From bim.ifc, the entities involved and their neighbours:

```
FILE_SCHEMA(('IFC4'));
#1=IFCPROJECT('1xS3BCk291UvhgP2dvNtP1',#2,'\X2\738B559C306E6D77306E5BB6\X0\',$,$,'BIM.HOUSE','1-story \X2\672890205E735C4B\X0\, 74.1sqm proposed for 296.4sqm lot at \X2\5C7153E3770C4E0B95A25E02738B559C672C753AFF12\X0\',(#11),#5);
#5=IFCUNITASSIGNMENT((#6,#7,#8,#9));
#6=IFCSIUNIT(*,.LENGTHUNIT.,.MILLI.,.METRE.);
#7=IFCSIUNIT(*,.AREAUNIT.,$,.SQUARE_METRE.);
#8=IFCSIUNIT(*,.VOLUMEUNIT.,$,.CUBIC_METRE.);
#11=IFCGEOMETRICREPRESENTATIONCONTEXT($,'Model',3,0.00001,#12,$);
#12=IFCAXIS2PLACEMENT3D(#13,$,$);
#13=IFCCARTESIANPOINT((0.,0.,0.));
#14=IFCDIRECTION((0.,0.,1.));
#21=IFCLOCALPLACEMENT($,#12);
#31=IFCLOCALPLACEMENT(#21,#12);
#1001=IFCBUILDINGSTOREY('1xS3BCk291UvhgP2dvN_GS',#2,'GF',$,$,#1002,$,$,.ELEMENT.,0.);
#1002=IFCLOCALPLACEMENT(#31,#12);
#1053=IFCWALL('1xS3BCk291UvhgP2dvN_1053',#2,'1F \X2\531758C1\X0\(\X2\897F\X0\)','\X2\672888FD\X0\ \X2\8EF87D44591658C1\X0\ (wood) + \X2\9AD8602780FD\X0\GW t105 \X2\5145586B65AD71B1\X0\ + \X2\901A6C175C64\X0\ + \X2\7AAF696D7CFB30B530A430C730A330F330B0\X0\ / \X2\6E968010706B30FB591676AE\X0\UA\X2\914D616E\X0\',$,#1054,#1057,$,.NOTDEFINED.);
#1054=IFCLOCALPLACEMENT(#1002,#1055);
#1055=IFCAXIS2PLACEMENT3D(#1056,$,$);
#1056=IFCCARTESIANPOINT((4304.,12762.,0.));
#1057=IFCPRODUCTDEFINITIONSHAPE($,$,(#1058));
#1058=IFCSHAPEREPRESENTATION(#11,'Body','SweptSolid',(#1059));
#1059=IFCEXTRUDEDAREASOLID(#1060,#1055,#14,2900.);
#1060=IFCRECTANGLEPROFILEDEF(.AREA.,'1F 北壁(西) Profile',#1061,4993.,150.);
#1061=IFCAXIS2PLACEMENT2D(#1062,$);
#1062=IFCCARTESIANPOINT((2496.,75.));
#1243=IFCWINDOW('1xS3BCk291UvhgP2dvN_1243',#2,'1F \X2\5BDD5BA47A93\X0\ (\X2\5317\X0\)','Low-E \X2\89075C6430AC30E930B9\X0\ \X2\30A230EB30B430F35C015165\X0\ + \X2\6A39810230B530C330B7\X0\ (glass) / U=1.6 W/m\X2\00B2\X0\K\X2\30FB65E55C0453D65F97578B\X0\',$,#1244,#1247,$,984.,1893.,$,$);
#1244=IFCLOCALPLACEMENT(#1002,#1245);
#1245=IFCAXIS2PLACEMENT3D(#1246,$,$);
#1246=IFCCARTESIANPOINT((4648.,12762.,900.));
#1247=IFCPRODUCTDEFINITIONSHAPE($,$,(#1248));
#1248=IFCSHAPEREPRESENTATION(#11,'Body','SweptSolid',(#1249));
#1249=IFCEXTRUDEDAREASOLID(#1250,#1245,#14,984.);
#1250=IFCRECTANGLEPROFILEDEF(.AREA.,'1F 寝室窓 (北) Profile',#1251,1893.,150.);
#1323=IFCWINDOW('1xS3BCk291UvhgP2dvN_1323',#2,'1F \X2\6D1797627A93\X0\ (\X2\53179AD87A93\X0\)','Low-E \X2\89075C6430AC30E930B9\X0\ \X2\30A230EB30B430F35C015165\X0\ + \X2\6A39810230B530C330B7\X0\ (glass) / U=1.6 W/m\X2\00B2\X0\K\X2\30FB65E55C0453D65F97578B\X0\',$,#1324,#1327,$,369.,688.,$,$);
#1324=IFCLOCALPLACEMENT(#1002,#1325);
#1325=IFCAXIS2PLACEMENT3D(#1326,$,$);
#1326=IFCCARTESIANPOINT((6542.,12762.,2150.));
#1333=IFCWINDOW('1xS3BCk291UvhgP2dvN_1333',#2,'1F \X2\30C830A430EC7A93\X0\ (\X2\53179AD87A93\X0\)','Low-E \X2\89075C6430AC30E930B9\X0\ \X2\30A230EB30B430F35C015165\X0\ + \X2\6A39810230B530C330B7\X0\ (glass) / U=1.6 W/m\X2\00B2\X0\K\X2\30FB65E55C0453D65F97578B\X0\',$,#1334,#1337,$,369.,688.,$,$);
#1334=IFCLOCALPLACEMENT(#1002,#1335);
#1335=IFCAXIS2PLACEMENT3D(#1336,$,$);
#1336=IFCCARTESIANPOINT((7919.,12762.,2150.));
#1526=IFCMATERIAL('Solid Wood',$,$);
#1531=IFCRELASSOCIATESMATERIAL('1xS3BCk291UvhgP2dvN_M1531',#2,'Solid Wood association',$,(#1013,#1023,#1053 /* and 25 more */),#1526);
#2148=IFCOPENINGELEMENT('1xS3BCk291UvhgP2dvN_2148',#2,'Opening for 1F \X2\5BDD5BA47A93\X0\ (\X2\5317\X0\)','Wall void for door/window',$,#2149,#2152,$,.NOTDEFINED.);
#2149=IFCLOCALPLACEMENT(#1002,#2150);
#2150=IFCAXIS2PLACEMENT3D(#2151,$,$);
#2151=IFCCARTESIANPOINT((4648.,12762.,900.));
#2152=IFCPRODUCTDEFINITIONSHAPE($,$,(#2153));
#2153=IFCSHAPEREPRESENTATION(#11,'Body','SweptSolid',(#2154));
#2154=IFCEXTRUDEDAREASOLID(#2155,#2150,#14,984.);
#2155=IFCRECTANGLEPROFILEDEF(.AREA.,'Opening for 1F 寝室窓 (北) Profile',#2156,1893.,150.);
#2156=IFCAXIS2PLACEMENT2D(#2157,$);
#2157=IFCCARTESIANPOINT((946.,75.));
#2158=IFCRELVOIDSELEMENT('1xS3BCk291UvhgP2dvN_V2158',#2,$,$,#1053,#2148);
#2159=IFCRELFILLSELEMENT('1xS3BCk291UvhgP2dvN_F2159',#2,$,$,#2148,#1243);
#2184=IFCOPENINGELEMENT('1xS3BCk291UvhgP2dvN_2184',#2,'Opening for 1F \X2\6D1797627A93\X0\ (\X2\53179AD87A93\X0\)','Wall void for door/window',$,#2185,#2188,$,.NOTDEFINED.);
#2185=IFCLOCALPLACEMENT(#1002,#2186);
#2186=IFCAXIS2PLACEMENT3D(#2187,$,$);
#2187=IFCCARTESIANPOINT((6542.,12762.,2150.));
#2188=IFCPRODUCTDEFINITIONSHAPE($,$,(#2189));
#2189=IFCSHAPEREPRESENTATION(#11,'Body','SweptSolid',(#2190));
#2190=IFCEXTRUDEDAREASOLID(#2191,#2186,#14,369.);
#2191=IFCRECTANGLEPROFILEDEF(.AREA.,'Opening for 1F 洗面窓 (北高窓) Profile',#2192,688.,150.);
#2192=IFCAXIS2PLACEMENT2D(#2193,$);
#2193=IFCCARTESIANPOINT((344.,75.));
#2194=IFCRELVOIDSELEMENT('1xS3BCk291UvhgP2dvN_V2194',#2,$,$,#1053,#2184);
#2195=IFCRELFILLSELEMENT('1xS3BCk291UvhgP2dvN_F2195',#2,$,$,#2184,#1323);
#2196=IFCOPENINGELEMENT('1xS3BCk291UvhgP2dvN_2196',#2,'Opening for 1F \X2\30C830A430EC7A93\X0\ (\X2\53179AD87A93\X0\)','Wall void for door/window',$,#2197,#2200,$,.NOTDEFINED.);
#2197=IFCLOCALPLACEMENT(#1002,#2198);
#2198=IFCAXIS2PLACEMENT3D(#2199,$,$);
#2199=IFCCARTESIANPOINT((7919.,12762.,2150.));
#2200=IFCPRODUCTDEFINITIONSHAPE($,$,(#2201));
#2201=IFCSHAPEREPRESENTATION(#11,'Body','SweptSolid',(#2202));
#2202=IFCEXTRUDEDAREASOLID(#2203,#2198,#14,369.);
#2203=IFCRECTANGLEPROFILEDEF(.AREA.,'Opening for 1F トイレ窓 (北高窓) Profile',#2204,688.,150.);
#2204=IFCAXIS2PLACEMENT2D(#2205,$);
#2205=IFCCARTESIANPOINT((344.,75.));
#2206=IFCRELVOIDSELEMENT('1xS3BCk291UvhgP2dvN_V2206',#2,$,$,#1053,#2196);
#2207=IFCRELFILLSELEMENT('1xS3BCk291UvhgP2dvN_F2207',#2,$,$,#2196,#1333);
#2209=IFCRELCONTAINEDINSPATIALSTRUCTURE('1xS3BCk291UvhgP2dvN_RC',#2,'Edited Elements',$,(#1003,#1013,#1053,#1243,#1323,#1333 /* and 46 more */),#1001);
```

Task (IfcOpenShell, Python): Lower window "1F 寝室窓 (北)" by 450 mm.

```python
import numpy as np
import ifcopenshell
import ifcopenshell.api.geometry
import ifcopenshell.util.placement
import ifcopenshell.util.unit

model = ifcopenshell.open("bim.ifc")
unit_scale = ifcopenshell.util.unit.calculate_unit_scale(model)

window = model.by_guid("1xS3BCk291UvhgP2dvN_1243")
opening = window.FillsVoids[0].RelatingOpeningElement
dz = -450.0

shift = np.array([0.0, 0.0, dz])
# The window is not placed relative to its opening, so move both.
for product in (opening, window):
    matrix = ifcopenshell.util.placement.get_local_placement(product.ObjectPlacement)
    matrix[:3, 3] += shift
    ifcopenshell.api.geometry.edit_object_placement(model, product=product, matrix=matrix, is_si=False)

print(f"moved by {dz * unit_scale:+.3f} m")

model.write("bim_v2.ifc")
```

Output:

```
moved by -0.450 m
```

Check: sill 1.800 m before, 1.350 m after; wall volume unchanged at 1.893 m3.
